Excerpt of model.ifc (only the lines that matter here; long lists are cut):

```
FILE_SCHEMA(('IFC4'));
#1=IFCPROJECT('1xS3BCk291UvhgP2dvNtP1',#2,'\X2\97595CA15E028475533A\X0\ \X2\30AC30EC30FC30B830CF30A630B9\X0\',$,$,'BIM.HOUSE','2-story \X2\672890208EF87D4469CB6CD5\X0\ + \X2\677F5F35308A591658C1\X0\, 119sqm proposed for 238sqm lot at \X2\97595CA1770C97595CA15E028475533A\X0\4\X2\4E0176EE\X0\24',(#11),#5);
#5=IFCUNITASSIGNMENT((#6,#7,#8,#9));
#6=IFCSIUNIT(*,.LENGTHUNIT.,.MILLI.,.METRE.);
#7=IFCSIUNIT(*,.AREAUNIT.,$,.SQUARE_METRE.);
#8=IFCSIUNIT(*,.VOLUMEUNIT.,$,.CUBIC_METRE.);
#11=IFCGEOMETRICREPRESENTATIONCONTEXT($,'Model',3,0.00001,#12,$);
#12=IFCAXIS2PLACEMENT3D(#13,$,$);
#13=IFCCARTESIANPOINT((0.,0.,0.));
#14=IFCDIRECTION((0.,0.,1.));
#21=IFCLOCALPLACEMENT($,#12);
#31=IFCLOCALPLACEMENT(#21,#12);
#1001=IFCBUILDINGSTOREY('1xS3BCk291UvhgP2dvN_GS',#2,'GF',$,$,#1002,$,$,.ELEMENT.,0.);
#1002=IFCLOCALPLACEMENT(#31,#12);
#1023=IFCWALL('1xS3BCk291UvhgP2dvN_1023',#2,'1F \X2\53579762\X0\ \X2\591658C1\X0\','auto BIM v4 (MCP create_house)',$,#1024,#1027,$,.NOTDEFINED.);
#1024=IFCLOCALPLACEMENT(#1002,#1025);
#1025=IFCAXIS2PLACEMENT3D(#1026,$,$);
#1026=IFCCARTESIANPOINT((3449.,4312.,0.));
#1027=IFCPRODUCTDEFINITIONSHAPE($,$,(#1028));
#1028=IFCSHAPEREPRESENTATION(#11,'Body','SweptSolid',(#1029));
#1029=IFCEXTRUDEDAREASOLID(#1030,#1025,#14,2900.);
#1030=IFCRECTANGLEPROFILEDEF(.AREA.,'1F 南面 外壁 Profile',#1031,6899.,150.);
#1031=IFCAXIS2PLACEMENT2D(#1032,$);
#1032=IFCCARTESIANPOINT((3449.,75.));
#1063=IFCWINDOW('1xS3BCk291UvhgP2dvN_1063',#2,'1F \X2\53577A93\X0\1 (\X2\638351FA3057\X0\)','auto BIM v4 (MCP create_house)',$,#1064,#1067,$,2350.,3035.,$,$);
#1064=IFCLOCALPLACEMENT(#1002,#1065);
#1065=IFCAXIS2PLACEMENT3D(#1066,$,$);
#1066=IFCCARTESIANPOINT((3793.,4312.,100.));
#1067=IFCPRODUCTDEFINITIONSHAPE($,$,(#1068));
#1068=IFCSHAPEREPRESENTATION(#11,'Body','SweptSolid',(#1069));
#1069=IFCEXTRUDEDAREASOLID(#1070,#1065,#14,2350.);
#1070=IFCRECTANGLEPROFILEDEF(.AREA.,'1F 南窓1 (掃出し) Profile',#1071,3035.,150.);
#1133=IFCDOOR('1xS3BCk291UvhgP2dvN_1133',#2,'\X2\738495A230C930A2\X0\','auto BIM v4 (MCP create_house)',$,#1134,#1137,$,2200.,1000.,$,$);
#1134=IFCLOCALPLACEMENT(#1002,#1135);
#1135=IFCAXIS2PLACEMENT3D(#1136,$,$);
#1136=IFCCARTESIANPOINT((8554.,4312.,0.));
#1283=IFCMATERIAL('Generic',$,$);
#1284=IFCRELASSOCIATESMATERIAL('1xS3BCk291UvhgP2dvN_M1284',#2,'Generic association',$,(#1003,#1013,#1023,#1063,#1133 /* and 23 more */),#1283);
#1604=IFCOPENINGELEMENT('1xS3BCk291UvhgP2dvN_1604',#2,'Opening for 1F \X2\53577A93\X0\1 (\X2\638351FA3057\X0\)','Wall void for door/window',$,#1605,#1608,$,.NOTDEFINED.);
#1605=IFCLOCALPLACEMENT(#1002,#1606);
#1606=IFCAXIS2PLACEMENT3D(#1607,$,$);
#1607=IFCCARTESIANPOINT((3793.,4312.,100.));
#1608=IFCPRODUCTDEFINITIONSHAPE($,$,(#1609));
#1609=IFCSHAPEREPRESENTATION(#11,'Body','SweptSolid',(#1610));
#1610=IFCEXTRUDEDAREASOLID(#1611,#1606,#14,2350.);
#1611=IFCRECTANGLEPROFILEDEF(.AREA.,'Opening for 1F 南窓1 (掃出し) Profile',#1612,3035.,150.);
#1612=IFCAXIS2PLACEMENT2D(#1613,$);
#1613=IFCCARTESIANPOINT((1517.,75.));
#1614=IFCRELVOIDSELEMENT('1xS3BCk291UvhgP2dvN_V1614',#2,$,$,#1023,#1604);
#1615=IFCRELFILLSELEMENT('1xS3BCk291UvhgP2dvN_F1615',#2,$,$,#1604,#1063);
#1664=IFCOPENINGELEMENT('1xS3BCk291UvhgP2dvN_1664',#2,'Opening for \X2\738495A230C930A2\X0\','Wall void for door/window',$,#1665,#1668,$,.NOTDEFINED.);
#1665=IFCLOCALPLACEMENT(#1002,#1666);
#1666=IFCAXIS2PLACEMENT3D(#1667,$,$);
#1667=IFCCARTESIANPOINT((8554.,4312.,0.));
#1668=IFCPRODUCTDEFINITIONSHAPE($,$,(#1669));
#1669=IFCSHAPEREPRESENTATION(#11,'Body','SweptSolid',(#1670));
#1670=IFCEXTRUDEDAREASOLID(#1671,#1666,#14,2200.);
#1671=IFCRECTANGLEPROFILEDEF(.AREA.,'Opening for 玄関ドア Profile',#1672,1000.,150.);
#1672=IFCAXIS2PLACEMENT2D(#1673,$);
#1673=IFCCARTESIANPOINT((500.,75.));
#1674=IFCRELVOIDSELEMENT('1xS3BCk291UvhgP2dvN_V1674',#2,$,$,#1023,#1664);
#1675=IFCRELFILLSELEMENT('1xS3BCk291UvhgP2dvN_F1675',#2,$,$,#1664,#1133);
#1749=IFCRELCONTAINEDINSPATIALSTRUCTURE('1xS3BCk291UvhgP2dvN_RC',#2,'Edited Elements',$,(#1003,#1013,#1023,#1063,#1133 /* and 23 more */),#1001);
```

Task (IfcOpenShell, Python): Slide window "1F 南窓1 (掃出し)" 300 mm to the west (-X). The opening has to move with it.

```python
import ifcopenshell
import ifcopenshell.api.geometry
import ifcopenshell.util.placement
import ifcopenshell.util.unit

model = ifcopenshell.open("model.ifc")
unit_scale = ifcopenshell.util.unit.calculate_unit_scale(model)

window = model.by_guid("1xS3BCk291UvhgP2dvN_1063")
opening = window.FillsVoids[0].RelatingOpeningElement
wall = opening.VoidsElements[0].RelatingBuildingElement

wall_matrix = ifcopenshell.util.placement.get_local_placement(wall.ObjectPlacement)
shift = wall_matrix[:3, 0] * -0.3 / unit_scale
before = ifcopenshell.util.placement.get_local_placement(window.ObjectPlacement)[:3, 3].copy()

# The window is not placed relative to its opening, so move both.
for product in (opening, window):
    matrix = ifcopenshell.util.placement.get_local_placement(product.ObjectPlacement)
    matrix[:3, 3] += shift
    ifcopenshell.api.geometry.edit_object_placement(model, product=product, matrix=matrix, is_si=False)

after = ifcopenshell.util.placement.get_local_placement(window.ObjectPlacement)[:3, 3]
print("window moved by", (after - before).round(3) + 0.0)

model.write("model_updated.ifc")
```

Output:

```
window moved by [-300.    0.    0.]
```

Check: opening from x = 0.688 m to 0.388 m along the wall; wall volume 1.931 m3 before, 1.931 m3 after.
